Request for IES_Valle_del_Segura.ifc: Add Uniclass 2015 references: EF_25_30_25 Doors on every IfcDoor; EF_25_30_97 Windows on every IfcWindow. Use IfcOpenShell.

First a look at what the model holds.

```python
import ifcopenshell

model = ifcopenshell.open("IES_Valle_del_Segura.ifc")
print(model.schema)
print("classifications:", [c.Name for c in model.by_type("IfcClassification")])
for ifc_class in ("IfcDoor", "IfcRoof", "IfcStair", "IfcWall", "IfcWindow"):
    print(ifc_class, len(model.by_type(ifc_class)))
```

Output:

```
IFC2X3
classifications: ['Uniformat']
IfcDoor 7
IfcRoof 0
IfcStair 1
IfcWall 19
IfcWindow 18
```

```python
import ifcopenshell
import ifcopenshell.api.classification

model = ifcopenshell.open("IES_Valle_del_Segura.ifc")

# IFC2X3 requires Source and Edition and has no link from the project to the system.
system = model.create_entity("IfcClassification", Source="NBS", Edition="2015", Name="Uniclass 2015")

codes = {
    "IfcDoor": ("EF_25_30_25", "Doors"),
    "IfcWindow": ("EF_25_30_97", "Windows"),
}
for ifc_class, (code, name) in codes.items():
    products = model.by_type(ifc_class)
    ifcopenshell.api.classification.add_reference(
        model, products=products, classification=system, identification=code, name=name
    )
    print(code, len(products))

model.write("IES_Valle_del_Segura_rev.ifc")
```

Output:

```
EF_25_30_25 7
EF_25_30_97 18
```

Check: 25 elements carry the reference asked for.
